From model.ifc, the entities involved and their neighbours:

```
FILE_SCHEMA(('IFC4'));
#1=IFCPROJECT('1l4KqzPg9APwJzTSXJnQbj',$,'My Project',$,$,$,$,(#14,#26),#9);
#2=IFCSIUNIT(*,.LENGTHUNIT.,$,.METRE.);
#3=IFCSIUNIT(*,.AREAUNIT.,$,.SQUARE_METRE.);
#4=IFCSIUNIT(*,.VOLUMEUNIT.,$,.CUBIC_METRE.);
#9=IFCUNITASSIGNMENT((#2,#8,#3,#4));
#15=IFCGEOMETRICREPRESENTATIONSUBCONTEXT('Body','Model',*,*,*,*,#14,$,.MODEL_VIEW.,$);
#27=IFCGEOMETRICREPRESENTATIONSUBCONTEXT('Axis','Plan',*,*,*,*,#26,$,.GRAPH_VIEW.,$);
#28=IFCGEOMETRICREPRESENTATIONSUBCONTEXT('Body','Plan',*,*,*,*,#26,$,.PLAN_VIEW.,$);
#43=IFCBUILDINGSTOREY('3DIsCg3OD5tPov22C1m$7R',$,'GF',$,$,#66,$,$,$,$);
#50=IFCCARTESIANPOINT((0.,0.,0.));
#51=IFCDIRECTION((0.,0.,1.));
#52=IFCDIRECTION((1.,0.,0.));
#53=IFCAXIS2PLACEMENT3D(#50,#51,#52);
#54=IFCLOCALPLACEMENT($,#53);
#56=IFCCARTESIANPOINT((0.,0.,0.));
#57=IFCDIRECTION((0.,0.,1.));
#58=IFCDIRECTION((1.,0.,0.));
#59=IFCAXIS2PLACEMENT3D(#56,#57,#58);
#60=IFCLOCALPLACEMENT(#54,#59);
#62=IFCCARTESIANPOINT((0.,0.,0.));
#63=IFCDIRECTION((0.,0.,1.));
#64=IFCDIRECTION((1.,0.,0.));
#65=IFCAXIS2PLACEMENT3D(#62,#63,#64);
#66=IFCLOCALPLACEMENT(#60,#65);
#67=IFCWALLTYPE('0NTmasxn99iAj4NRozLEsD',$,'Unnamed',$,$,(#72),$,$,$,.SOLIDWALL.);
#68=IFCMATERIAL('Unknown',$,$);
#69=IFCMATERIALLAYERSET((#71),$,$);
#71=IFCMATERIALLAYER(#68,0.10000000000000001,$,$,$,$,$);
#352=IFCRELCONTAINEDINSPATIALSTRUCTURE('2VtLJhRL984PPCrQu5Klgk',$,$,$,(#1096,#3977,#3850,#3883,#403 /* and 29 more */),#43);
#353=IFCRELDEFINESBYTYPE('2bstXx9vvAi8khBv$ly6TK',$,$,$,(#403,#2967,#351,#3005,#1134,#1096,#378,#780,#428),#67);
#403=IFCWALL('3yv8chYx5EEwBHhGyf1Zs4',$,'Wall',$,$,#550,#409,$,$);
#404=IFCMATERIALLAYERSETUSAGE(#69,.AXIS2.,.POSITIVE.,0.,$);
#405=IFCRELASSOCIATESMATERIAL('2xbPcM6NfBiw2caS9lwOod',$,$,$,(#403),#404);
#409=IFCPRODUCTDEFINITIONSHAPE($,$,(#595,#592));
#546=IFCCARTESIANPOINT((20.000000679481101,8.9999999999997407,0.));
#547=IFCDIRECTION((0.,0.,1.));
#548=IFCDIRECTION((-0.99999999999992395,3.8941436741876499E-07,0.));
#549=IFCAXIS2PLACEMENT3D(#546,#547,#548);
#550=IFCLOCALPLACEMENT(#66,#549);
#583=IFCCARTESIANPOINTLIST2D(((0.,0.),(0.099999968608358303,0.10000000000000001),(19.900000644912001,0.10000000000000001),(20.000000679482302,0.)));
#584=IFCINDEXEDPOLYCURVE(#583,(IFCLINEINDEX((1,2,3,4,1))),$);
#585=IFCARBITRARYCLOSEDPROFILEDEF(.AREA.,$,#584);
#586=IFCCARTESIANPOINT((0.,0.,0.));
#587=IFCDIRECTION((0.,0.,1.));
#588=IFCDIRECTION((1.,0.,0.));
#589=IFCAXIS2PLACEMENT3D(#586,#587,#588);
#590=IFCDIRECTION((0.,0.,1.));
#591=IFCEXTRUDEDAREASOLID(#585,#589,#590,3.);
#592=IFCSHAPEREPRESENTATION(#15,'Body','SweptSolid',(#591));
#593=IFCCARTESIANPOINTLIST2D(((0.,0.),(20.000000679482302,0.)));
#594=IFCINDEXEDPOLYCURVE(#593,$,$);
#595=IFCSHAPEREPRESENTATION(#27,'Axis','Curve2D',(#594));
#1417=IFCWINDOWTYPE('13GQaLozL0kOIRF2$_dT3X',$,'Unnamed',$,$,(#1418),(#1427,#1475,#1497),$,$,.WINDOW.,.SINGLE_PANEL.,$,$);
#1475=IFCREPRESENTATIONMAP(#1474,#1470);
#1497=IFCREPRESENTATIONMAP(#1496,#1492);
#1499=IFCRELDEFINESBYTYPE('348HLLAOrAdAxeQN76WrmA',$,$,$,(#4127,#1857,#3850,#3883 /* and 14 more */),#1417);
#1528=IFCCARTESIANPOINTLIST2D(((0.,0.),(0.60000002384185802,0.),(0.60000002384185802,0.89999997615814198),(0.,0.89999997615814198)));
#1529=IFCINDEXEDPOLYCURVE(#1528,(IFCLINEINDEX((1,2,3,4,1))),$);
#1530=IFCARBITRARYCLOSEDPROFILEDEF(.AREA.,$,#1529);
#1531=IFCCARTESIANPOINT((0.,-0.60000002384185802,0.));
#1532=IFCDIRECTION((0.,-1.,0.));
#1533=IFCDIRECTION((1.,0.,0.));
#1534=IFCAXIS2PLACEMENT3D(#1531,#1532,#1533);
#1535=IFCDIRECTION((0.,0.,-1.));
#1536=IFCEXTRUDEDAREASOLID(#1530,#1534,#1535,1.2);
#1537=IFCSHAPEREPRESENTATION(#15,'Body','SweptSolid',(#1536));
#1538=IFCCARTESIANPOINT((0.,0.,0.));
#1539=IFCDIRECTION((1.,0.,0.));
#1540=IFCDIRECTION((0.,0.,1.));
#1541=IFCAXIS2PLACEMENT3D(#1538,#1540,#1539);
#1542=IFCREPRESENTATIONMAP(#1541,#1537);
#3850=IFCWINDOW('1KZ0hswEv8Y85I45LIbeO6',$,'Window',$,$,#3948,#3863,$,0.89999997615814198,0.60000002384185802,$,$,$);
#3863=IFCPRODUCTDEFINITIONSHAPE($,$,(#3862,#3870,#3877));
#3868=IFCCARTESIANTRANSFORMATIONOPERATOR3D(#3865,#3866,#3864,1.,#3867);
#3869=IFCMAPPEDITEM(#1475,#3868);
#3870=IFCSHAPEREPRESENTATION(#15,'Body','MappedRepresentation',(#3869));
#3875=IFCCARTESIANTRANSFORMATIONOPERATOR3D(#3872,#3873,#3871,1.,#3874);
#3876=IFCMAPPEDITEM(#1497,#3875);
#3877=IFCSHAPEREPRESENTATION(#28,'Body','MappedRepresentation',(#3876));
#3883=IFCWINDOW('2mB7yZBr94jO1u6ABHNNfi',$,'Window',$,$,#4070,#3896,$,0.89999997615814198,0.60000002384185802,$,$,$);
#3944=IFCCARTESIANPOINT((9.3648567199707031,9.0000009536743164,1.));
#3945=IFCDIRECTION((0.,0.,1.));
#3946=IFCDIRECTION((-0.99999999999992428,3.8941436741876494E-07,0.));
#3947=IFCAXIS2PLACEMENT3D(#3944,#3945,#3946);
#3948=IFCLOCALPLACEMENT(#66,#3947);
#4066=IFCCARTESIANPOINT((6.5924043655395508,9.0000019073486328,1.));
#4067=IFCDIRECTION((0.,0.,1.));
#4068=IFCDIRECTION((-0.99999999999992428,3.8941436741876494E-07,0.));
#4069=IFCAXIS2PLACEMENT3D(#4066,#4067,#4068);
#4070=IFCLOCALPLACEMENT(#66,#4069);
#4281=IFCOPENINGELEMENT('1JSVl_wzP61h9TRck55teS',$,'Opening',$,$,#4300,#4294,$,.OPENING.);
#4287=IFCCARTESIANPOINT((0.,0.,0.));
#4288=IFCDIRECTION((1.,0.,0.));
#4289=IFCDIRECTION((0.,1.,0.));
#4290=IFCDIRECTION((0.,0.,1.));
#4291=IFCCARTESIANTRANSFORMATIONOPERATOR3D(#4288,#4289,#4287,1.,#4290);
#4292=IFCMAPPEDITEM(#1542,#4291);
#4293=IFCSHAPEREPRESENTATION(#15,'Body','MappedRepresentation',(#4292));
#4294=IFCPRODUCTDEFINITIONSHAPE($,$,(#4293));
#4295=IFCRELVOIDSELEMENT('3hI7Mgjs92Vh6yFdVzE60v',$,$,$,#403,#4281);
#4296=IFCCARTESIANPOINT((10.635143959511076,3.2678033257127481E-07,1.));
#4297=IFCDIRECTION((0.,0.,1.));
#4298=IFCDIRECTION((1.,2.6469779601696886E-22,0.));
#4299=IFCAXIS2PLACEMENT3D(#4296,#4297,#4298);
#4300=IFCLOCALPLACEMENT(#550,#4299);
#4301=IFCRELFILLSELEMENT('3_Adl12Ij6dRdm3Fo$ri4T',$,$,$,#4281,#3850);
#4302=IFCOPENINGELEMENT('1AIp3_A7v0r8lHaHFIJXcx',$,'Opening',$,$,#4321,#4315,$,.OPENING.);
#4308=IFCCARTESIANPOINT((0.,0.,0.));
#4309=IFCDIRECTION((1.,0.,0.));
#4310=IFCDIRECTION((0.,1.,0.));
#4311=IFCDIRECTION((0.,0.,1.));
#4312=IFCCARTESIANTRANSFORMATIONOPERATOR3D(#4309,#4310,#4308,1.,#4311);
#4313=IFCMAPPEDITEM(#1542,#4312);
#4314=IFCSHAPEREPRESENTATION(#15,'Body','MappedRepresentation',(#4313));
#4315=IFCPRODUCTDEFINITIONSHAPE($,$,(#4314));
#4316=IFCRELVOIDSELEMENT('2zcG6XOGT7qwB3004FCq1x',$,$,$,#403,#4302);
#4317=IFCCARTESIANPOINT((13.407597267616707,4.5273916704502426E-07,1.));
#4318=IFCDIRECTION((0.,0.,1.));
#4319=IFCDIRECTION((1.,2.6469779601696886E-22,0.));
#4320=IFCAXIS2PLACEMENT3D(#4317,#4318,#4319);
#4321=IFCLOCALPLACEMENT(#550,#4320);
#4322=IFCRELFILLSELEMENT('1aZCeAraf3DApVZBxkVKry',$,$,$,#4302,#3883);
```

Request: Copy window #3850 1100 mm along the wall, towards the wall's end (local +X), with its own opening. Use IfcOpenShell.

```python
import ifcopenshell
import ifcopenshell.api.feature
import ifcopenshell.api.geometry
import ifcopenshell.api.root
import ifcopenshell.geom
import ifcopenshell.util.element
import ifcopenshell.util.placement
import ifcopenshell.util.shape

model = ifcopenshell.open("model.ifc")
settings = ifcopenshell.geom.settings()


def volume(element):
    """Net volume in cubic metres, openings subtracted."""
    shape = ifcopenshell.geom.create_shape(settings, element)
    return ifcopenshell.util.shape.get_volume(shape.geometry)


window = model.by_id(3850)
opening = window.FillsVoids[0].RelatingOpeningElement
wall = opening.VoidsElements[0].RelatingBuildingElement
before = volume(wall)
shift = ifcopenshell.util.placement.get_local_placement(wall.ObjectPlacement)[:3, 0] * 1.1

# copy_class copies the void relationship, type, container and properties, but no geometry.
new_opening = ifcopenshell.api.root.copy_class(model, product=opening)
new_opening.Representation = ifcopenshell.util.element.copy_deep(
    model, opening.Representation, exclude=["IfcGeometricRepresentationContext", "IfcRepresentationMap"]
)
new_window = ifcopenshell.api.root.copy_class(model, product=window)
new_window.Representation = ifcopenshell.util.element.copy_deep(
    model, window.Representation, exclude=["IfcGeometricRepresentationContext", "IfcRepresentationMap"]
)
ifcopenshell.api.feature.add_filling(model, opening=new_opening, element=new_window)

for old, new in ((opening, new_opening), (window, new_window)):
    matrix = ifcopenshell.util.placement.get_local_placement(old.ObjectPlacement)
    matrix[:3, 3] += shift
    ifcopenshell.api.geometry.edit_object_placement(model, product=new, matrix=matrix, is_si=False)

after = volume(wall)

print(f"wall volume {before:.3f} -> {after:.3f} m3")

model.write("model-out.ifc")
```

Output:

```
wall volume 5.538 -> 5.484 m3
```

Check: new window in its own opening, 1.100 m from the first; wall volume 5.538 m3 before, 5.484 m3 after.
